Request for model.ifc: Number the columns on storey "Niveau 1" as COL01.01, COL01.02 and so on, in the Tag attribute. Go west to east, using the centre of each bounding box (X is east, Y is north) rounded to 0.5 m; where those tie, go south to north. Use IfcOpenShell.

First a look at what the model holds.

```python
import ifcopenshell
import ifcopenshell.util.element
import ifcopenshell.util.placement

model = ifcopenshell.open("model.ifc")
print(model.schema)
storey = next(s for s in model.by_type("IfcBuildingStorey") if s.Name == "Niveau 1")
columns = [e for e in ifcopenshell.util.element.get_decomposition(storey) if e.is_a("IfcColumn")]
for e in sorted(columns, key=lambda e: e.id()):
    origin = ifcopenshell.util.placement.get_local_placement(e.ObjectPlacement)[:3, 3]
    print(e.id(), e.Tag, e.Name, origin.round(2) + 0.0, sep=" | ")
```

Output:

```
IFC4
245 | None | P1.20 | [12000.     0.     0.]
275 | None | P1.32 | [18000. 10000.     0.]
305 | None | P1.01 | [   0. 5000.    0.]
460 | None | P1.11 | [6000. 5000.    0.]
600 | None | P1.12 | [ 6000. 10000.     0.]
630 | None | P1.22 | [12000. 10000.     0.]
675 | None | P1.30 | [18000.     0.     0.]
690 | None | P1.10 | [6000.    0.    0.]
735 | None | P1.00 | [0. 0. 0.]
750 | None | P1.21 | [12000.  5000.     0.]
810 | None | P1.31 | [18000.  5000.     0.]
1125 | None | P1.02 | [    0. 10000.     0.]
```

```python
import ifcopenshell
import ifcopenshell.geom
import ifcopenshell.util.element
import ifcopenshell.util.shape

model = ifcopenshell.open("model.ifc")
settings = ifcopenshell.geom.settings()
settings.set("use-world-coords", True)


def centre(element):
    shape = ifcopenshell.geom.create_shape(settings, element)
    return ifcopenshell.util.shape.get_bbox_centroid(shape.geometry)


storey = next(s for s in model.by_type("IfcBuildingStorey") if s.Name == "Niveau 1")
columns = [e for e in ifcopenshell.util.element.get_decomposition(storey) if e.is_a("IfcColumn")]

# Insertion points can sit at a corner or the storey origin, so sort by the geometry (in metres).
centres = {e: centre(e) for e in columns}
columns.sort(key=lambda e: (round(centres[e][0] / 0.5), centres[e][1]))

for i, e in enumerate(columns, start=1):
    number = f"COL01.{i:02d}"
    e.Tag = number
    print(e.id(), number)

model.write("model_v2.ifc")
```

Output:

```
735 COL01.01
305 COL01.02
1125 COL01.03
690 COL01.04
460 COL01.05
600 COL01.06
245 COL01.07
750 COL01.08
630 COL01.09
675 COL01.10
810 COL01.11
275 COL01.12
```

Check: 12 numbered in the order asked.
